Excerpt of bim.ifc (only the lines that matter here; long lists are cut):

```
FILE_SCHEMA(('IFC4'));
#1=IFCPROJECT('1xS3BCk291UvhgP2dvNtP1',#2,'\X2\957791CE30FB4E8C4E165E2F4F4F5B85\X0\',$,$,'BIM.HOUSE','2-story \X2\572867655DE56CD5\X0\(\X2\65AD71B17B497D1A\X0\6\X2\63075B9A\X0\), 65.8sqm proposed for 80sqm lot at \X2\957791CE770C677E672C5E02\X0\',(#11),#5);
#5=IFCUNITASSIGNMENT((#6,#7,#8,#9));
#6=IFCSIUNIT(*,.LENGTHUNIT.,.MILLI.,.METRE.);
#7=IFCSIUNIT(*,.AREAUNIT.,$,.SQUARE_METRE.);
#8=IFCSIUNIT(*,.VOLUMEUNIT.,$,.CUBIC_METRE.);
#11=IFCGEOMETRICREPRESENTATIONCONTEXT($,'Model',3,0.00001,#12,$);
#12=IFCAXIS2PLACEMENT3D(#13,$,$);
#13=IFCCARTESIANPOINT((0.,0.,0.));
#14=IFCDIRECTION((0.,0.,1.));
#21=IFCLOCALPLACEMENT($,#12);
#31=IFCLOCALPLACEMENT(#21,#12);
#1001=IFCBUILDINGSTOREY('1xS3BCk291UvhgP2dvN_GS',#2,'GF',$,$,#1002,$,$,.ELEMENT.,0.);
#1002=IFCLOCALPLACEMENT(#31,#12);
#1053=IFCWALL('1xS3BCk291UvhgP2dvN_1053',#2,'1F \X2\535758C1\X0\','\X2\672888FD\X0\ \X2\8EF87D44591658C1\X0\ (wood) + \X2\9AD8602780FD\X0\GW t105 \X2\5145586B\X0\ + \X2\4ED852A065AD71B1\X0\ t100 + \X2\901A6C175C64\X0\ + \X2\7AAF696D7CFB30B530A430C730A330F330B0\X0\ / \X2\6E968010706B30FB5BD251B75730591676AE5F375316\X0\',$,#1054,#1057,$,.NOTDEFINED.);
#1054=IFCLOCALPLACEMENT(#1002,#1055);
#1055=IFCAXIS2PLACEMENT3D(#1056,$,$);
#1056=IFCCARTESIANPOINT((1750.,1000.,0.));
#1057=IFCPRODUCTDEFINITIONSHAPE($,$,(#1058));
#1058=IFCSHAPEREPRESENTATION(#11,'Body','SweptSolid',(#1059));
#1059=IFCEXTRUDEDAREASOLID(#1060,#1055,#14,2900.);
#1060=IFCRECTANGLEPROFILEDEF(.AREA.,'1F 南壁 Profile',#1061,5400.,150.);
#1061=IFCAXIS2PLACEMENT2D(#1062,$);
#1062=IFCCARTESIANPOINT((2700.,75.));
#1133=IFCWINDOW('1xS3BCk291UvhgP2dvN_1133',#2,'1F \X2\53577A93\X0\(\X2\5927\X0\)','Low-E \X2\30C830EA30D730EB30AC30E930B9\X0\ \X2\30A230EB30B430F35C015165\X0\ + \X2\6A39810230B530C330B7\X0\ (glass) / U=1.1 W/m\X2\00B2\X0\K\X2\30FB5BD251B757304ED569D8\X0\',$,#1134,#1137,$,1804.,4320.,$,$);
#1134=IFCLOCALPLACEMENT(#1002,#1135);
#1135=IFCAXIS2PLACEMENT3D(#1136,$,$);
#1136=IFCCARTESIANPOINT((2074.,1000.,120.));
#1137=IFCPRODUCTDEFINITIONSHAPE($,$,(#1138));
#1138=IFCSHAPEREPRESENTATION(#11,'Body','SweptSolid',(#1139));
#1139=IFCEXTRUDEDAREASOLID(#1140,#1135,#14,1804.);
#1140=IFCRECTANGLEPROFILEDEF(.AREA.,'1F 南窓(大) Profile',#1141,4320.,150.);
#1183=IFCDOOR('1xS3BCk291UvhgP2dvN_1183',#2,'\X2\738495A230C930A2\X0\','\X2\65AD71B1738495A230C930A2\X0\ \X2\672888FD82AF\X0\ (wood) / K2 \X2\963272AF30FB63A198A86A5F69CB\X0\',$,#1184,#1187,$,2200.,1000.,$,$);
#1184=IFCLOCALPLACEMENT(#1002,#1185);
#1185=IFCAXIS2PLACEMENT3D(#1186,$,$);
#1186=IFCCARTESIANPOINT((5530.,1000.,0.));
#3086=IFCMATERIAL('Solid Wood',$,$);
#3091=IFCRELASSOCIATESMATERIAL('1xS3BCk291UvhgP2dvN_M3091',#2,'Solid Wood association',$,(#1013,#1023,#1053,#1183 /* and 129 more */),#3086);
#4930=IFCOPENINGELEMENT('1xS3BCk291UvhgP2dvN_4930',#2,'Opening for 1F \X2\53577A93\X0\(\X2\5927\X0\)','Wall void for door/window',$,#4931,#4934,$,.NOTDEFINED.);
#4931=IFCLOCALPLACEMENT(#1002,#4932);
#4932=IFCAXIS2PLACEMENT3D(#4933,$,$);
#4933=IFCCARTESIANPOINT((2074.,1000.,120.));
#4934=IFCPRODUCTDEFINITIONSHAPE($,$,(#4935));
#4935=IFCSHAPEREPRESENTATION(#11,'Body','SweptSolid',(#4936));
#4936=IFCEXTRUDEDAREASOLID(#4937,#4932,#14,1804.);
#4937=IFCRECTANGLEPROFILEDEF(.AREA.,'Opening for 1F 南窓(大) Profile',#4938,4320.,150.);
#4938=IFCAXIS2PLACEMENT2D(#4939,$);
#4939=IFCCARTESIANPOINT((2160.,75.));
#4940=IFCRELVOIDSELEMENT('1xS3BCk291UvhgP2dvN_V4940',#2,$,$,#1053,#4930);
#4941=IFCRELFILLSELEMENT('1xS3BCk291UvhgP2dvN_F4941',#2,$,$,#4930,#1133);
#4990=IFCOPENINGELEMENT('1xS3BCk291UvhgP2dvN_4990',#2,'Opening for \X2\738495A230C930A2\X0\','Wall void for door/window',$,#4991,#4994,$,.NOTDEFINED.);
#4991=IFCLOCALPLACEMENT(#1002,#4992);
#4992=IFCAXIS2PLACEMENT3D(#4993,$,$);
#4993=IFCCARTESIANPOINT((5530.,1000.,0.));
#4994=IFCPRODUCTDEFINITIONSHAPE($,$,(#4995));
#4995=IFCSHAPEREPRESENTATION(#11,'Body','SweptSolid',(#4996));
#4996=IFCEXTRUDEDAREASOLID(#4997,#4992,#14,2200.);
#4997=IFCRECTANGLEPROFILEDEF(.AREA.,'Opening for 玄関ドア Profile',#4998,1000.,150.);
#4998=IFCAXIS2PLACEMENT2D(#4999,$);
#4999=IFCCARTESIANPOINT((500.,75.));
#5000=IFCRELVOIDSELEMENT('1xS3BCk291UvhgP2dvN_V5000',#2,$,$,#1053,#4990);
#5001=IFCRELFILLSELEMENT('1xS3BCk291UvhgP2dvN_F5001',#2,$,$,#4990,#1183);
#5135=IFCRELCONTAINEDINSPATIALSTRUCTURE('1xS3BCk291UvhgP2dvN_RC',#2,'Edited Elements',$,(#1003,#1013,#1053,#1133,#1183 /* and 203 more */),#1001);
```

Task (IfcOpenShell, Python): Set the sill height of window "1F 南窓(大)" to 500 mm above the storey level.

```python
import numpy as np
import ifcopenshell
import ifcopenshell.api.geometry
import ifcopenshell.geom
import ifcopenshell.util.element
import ifcopenshell.util.placement
import ifcopenshell.util.shape
import ifcopenshell.util.unit

model = ifcopenshell.open("bim.ifc")
unit_scale = ifcopenshell.util.unit.calculate_unit_scale(model)

window = model.by_guid("1xS3BCk291UvhgP2dvN_1133")
opening = window.FillsVoids[0].RelatingOpeningElement
storey = ifcopenshell.util.element.get_container(window, ifc_class="IfcBuildingStorey")
level = ifcopenshell.util.placement.get_local_placement(storey.ObjectPlacement)[2, 3]

# The opening's origin need not be at the sill, so measure its lowest point.
shape = ifcopenshell.geom.create_shape(ifcopenshell.geom.settings(), opening)
bottom = ifcopenshell.util.shape.get_shape_bottom_elevation(shape, shape.geometry) / unit_scale
dz = level + 0.5 / unit_scale - bottom

shift = np.array([0.0, 0.0, dz])
# The window is not placed relative to its opening, so move both.
for product in (opening, window):
    matrix = ifcopenshell.util.placement.get_local_placement(product.ObjectPlacement)
    matrix[:3, 3] += shift
    ifcopenshell.api.geometry.edit_object_placement(model, product=product, matrix=matrix, is_si=False)

print(f"moved by {dz * unit_scale:+.3f} m")

model.write("bim_updated.ifc")
```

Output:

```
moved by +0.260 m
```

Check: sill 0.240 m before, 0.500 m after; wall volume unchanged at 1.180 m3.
